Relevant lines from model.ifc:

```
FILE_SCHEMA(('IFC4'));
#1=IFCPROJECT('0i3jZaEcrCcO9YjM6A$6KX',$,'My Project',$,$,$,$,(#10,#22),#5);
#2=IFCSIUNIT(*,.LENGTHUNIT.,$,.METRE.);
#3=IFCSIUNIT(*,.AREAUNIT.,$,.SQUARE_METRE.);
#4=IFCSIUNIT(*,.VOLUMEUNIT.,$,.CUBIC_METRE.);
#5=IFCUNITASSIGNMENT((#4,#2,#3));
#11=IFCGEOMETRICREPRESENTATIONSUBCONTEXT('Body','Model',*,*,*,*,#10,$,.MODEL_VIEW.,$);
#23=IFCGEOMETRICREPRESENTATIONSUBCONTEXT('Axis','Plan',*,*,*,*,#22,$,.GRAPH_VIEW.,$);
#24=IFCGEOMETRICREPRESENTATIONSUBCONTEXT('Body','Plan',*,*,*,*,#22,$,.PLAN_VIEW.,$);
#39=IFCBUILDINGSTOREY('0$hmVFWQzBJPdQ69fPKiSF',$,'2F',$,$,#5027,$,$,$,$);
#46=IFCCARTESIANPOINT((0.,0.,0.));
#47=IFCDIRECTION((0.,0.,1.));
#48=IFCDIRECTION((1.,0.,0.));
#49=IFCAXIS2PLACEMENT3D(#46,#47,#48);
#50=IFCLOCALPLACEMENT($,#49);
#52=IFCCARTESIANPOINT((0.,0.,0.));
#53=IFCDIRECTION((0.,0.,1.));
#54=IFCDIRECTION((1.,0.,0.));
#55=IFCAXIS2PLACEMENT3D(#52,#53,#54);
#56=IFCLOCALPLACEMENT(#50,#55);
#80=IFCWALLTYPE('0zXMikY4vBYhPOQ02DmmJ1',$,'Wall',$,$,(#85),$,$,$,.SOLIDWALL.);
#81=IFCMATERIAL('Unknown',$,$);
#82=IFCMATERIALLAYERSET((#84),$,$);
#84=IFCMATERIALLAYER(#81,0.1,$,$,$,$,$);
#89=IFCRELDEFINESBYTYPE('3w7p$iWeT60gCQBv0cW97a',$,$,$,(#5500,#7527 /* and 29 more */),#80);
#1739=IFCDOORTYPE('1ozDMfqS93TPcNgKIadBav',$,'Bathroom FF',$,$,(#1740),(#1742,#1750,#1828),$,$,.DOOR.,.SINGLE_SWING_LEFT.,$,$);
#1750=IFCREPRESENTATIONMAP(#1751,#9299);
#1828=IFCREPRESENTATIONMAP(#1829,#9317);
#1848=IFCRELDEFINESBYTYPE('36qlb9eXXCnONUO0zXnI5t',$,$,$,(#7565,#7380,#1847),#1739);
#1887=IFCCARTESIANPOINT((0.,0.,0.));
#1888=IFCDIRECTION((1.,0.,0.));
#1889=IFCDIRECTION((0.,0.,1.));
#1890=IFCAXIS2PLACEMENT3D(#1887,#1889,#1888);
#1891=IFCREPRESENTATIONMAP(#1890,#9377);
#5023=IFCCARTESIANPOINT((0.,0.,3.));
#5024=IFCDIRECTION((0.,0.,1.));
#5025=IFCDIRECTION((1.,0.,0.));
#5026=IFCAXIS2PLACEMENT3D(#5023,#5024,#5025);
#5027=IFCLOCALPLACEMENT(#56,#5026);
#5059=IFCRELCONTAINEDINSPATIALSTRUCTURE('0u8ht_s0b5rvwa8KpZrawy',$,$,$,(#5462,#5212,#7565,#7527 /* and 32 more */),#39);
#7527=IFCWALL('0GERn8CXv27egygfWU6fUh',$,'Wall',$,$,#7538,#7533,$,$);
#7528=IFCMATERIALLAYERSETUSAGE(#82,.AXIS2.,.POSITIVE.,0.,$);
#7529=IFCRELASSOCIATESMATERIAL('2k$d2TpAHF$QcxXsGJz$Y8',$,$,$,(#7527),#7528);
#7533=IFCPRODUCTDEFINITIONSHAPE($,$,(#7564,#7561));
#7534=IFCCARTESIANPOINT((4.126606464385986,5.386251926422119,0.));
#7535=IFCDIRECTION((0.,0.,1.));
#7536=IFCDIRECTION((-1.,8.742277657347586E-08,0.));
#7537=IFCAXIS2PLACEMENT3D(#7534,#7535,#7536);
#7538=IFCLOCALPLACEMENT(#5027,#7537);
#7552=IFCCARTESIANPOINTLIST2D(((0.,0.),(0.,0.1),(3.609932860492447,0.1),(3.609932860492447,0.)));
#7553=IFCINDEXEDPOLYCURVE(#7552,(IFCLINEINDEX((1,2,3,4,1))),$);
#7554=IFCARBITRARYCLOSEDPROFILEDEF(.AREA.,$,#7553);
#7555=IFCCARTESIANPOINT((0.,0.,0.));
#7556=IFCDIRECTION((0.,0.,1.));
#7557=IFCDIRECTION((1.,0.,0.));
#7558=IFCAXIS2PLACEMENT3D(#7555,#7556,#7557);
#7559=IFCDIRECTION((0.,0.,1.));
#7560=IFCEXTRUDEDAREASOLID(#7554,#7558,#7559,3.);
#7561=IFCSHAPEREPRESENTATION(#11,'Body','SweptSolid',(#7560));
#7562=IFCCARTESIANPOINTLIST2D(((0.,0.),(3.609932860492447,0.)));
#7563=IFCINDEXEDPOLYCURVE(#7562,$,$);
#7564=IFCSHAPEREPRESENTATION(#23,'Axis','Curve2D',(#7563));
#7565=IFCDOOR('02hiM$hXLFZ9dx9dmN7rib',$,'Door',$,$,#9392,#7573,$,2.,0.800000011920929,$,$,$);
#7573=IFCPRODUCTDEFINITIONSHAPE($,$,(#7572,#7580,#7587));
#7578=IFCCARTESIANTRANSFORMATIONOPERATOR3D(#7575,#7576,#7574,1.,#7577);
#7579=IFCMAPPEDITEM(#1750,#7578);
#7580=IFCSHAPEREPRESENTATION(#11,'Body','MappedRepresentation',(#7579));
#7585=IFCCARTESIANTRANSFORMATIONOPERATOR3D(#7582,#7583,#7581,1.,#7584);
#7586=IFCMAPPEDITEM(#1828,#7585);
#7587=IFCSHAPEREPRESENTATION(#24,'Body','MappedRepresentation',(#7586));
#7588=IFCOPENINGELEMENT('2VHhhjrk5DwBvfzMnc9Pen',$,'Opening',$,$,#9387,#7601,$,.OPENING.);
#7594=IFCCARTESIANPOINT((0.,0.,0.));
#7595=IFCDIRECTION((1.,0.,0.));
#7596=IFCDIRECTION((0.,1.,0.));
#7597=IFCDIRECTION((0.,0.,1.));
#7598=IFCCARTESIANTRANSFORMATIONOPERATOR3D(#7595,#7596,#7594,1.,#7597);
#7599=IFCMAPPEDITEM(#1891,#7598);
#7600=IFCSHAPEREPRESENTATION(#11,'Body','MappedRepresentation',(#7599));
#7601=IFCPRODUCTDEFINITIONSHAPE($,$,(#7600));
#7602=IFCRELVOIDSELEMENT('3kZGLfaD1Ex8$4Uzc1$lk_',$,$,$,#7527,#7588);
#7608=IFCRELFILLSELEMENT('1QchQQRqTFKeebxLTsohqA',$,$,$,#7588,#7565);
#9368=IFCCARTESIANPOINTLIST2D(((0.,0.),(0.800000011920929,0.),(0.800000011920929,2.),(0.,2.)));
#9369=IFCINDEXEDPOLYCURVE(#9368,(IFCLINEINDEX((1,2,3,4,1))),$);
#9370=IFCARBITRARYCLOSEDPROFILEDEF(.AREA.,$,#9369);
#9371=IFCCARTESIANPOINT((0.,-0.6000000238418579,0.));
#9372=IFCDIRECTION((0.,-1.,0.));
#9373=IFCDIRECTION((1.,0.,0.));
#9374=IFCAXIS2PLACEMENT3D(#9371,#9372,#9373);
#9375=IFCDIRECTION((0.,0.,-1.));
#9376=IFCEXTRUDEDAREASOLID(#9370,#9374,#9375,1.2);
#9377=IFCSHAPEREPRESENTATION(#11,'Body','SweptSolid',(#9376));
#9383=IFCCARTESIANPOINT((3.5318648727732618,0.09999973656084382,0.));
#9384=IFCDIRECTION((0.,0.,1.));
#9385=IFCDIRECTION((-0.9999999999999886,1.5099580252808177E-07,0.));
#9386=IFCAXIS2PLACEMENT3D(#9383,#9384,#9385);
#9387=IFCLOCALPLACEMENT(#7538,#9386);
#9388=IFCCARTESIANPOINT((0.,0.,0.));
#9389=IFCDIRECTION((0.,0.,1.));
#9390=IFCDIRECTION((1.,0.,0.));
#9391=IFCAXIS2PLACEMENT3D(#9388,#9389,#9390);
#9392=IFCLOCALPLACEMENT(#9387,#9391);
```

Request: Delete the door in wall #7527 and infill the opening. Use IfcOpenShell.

```python
import ifcopenshell
import ifcopenshell.api.feature
import ifcopenshell.api.root
import ifcopenshell.geom
import ifcopenshell.util.shape

model = ifcopenshell.open("model.ifc")
settings = ifcopenshell.geom.settings()


def volume(element):
    """Net volume in cubic metres, openings subtracted."""
    shape = ifcopenshell.geom.create_shape(settings, element)
    return ifcopenshell.util.shape.get_volume(shape.geometry)


door = model.by_id(7565)
opening = door.FillsVoids[0].RelatingOpeningElement
wall = opening.VoidsElements[0].RelatingBuildingElement
before = volume(wall)

ifcopenshell.api.root.remove_product(model, product=door)
ifcopenshell.api.feature.remove_feature(model, feature=opening)

after = volume(wall)

print(f"wall volume {before:.3f} -> {after:.3f} m3")

model.write("model-out.ifc")
```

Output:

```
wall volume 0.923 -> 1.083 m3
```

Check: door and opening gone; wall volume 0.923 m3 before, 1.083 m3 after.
